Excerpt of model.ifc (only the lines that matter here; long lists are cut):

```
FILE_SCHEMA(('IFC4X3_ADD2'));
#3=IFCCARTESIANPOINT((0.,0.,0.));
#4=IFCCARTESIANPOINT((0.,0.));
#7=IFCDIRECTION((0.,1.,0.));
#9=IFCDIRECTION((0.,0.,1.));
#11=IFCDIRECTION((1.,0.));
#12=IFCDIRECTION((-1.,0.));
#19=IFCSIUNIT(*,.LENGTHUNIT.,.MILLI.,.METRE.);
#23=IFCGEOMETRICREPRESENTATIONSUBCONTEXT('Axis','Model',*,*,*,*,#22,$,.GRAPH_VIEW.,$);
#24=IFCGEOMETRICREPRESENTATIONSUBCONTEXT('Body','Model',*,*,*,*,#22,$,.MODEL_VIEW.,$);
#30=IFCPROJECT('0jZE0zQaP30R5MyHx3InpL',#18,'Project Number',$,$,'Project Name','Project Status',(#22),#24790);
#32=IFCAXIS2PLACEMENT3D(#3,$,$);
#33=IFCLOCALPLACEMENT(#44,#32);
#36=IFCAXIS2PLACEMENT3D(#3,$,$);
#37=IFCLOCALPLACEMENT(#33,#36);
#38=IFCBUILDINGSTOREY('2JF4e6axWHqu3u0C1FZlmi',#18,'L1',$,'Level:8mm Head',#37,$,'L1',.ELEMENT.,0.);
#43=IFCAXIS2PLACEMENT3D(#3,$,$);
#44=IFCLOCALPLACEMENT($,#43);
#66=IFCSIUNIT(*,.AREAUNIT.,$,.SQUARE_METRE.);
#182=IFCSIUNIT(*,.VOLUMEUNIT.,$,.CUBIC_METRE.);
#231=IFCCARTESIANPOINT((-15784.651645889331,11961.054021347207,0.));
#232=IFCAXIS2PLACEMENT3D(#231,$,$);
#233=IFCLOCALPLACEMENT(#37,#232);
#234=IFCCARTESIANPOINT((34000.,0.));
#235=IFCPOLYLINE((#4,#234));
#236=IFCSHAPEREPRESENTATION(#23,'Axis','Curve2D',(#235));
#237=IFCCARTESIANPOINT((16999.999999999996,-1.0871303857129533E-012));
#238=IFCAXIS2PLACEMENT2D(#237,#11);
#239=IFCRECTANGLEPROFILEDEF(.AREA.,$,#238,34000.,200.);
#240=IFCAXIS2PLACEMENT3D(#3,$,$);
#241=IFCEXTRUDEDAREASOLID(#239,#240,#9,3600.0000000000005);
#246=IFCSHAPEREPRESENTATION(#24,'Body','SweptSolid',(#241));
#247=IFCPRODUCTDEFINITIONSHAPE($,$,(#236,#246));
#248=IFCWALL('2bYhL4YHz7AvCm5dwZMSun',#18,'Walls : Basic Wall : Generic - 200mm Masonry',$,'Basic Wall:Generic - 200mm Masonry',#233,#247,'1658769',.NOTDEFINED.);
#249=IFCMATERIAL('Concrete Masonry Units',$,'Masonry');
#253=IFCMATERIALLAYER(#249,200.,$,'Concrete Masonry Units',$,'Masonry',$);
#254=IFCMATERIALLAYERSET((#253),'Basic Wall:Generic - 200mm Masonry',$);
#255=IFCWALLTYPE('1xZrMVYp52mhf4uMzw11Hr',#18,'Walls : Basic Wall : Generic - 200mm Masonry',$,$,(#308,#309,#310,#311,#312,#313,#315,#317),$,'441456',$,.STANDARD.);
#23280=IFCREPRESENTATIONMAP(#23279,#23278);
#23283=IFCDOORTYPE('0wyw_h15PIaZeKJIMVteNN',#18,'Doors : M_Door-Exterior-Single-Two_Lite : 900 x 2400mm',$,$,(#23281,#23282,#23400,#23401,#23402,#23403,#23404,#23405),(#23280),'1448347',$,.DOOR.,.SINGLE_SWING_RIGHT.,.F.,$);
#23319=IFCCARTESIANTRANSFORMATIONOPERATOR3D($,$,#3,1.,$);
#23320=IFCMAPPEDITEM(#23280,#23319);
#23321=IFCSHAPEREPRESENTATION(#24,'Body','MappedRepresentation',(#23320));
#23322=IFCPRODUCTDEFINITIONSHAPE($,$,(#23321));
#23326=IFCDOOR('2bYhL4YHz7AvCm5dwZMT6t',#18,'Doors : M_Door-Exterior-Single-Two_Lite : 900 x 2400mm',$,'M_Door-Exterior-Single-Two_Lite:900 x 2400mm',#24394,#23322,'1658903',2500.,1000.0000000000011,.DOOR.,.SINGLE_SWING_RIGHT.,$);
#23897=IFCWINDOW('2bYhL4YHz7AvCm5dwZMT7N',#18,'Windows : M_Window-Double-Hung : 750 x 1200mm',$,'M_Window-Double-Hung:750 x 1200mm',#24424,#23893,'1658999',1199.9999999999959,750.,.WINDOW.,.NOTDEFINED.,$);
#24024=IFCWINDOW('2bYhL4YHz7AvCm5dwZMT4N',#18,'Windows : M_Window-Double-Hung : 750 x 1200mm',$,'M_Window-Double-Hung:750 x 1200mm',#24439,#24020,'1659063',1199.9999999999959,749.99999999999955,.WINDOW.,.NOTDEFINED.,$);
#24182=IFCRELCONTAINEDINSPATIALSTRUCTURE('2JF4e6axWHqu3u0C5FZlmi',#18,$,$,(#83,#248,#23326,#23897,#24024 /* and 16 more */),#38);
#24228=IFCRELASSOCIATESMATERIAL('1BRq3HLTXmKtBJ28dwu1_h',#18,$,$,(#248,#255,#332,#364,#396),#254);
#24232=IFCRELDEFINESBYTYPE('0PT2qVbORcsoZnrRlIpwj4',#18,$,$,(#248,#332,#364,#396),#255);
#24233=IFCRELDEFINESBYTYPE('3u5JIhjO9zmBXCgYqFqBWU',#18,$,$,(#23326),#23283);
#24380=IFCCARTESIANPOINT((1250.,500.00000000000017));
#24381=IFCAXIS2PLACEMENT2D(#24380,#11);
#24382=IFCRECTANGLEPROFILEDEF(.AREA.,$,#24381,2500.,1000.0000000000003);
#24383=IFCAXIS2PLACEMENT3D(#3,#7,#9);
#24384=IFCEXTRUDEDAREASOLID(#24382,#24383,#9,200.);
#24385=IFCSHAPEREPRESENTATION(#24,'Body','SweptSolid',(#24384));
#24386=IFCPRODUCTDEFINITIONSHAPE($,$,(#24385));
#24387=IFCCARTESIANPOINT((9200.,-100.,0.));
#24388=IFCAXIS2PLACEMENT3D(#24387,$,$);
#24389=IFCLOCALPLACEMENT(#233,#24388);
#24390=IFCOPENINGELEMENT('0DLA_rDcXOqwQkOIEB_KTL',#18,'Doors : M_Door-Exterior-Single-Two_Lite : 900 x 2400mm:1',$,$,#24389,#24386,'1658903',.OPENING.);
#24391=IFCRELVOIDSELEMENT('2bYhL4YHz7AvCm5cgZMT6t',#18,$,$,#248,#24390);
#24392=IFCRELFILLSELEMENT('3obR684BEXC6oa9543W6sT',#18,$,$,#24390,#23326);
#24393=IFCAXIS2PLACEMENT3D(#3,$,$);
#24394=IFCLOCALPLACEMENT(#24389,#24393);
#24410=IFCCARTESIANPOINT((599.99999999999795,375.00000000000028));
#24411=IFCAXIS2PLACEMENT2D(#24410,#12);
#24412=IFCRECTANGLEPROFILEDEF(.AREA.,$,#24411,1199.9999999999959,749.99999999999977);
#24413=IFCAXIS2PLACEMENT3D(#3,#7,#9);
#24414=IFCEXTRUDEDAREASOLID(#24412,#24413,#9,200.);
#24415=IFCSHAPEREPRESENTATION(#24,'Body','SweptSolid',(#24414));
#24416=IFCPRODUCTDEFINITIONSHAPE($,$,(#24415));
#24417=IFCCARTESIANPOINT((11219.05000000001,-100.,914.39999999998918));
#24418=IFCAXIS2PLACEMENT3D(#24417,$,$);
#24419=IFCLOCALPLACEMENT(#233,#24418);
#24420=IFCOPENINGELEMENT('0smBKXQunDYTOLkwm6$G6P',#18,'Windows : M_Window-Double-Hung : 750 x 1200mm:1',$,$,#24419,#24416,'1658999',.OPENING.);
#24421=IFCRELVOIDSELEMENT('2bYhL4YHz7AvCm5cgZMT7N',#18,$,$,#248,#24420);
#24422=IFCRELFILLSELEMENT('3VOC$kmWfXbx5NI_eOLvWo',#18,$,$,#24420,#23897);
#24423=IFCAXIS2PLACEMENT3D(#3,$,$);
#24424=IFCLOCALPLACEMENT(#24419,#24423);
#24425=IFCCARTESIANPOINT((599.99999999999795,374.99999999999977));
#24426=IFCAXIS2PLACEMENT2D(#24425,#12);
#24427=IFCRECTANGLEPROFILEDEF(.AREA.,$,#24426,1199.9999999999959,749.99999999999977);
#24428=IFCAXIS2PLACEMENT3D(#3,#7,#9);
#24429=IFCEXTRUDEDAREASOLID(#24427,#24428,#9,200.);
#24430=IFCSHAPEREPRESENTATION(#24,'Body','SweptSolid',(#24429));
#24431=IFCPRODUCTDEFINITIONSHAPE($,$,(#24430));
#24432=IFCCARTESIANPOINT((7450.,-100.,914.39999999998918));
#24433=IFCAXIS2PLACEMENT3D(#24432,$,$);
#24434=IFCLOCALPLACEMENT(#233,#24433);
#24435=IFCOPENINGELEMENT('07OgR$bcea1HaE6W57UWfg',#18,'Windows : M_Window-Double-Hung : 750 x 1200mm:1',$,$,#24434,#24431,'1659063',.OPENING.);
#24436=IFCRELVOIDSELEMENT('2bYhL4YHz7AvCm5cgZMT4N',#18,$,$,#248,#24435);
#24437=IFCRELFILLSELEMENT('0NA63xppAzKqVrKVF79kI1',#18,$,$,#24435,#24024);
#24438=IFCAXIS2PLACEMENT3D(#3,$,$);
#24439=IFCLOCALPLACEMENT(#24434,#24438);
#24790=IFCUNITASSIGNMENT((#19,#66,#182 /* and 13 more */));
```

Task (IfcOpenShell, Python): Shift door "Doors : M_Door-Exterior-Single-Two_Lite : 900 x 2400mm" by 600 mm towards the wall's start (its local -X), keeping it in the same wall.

```python
import ifcopenshell
import ifcopenshell.api.geometry
import ifcopenshell.util.placement

model = ifcopenshell.open("model.ifc")

door = model.by_id(23326)
opening = door.FillsVoids[0].RelatingOpeningElement
wall = opening.VoidsElements[0].RelatingBuildingElement

wall_matrix = ifcopenshell.util.placement.get_local_placement(wall.ObjectPlacement)
shift = wall_matrix[:3, 0] * -600.0
before = ifcopenshell.util.placement.get_local_placement(door.ObjectPlacement)[:3, 3].copy()

# The door is placed relative to its opening, so it follows when the opening moves.
matrix = ifcopenshell.util.placement.get_local_placement(opening.ObjectPlacement)
matrix[:3, 3] += shift
ifcopenshell.api.geometry.edit_object_placement(
    model, product=opening, matrix=matrix, is_si=False, should_transform_children=True
)

after = ifcopenshell.util.placement.get_local_placement(door.ObjectPlacement)[:3, 3]
print("door moved by", (after - before).round(3) + 0.0)

model.write("model_rev.ifc")
```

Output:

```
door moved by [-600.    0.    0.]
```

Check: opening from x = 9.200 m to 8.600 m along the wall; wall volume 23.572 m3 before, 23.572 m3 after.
